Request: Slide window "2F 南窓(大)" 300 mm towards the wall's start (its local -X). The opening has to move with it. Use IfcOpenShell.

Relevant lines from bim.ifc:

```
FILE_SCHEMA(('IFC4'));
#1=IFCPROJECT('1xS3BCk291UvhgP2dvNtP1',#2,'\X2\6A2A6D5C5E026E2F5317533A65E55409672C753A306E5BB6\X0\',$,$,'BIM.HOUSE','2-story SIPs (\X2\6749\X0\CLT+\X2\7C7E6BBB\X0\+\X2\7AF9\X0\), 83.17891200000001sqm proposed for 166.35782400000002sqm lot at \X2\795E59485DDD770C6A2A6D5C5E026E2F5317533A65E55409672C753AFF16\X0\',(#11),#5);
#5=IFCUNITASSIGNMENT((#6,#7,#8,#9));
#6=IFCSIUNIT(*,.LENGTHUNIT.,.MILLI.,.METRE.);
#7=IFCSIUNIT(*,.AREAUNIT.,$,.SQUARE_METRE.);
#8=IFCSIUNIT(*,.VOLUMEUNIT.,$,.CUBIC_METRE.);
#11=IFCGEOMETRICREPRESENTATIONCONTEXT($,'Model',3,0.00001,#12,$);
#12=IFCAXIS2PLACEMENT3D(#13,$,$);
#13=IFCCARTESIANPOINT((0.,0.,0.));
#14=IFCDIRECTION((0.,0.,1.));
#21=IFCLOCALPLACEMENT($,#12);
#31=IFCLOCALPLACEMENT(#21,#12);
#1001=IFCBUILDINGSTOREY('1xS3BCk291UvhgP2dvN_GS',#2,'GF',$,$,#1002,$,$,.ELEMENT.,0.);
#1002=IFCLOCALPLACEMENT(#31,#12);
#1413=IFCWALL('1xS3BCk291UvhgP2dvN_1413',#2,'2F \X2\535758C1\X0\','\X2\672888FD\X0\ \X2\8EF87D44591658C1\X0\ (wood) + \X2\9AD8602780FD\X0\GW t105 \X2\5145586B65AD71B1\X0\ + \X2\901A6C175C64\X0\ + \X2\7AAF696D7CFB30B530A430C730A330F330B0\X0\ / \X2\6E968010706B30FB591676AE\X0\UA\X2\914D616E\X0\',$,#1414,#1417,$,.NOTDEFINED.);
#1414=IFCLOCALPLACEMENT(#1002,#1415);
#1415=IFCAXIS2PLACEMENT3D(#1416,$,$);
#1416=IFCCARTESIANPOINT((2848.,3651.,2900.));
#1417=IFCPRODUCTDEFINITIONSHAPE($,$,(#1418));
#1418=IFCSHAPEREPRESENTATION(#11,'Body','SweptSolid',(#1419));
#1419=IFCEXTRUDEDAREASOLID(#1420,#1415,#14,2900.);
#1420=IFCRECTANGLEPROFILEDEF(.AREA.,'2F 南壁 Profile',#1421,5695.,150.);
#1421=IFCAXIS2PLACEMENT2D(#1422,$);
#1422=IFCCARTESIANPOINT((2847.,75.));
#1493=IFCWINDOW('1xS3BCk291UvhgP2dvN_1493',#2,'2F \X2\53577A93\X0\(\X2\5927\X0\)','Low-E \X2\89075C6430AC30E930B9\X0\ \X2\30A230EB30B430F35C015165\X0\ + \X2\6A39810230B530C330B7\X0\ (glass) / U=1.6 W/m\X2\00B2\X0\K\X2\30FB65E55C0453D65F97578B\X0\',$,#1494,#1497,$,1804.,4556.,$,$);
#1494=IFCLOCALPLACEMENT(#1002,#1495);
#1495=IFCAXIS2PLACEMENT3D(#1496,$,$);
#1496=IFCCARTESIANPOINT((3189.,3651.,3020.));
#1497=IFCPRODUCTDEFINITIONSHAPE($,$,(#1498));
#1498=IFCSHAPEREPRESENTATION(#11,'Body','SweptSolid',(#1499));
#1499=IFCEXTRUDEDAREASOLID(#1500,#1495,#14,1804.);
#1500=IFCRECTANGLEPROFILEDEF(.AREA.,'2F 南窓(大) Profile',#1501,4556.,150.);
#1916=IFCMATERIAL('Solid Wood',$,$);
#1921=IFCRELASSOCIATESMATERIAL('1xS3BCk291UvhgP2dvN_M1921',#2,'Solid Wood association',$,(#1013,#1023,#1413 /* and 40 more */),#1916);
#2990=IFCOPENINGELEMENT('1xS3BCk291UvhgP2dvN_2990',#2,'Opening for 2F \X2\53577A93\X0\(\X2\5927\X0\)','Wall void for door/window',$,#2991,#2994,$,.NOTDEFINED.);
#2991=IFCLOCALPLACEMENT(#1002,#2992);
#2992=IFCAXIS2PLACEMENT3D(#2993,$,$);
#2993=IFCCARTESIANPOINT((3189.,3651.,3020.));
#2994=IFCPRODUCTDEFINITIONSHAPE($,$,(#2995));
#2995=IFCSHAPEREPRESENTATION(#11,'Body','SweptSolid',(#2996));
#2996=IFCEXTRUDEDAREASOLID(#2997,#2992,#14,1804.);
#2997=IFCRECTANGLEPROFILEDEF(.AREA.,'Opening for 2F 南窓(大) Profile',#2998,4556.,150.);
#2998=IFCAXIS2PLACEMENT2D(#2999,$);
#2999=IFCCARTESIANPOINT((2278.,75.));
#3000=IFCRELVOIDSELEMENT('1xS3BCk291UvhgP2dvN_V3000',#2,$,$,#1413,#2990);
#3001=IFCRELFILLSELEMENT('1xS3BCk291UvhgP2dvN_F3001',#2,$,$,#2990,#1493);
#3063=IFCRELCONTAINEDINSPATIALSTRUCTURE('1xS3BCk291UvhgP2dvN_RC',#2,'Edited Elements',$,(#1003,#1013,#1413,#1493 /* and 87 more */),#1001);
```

```python
import ifcopenshell
import ifcopenshell.api.geometry
import ifcopenshell.util.placement
import ifcopenshell.util.unit

model = ifcopenshell.open("bim.ifc")
unit_scale = ifcopenshell.util.unit.calculate_unit_scale(model)

window = model.by_guid("1xS3BCk291UvhgP2dvN_1493")
opening = window.FillsVoids[0].RelatingOpeningElement
wall = opening.VoidsElements[0].RelatingBuildingElement

wall_matrix = ifcopenshell.util.placement.get_local_placement(wall.ObjectPlacement)
shift = wall_matrix[:3, 0] * -0.3 / unit_scale
before = ifcopenshell.util.placement.get_local_placement(window.ObjectPlacement)[:3, 3].copy()

# The window is not placed relative to its opening, so move both.
for product in (opening, window):
    matrix = ifcopenshell.util.placement.get_local_placement(product.ObjectPlacement)
    matrix[:3, 3] += shift
    ifcopenshell.api.geometry.edit_object_placement(model, product=product, matrix=matrix, is_si=False)

after = ifcopenshell.util.placement.get_local_placement(window.ObjectPlacement)[:3, 3]
print("window moved by", (after - before).round(3) + 0.0)

model.write("bim_edited.ifc")
```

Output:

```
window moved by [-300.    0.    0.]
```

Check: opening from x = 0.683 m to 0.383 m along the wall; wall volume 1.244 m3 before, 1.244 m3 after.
